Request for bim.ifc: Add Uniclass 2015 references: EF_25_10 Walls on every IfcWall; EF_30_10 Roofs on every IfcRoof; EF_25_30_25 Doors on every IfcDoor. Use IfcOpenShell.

First a look at what the model holds.

```python
import ifcopenshell

model = ifcopenshell.open("bim.ifc")
print(model.schema)
print("classifications:", [c.Name for c in model.by_type("IfcClassification")])
for ifc_class in ("IfcDoor", "IfcRoof", "IfcStair", "IfcWall", "IfcWindow"):
    print(ifc_class, len(model.by_type(ifc_class)))
```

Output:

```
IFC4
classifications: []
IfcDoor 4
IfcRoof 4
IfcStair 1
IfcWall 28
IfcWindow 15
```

```python
import ifcopenshell
import ifcopenshell.api.classification

model = ifcopenshell.open("bim.ifc")

system = ifcopenshell.api.classification.add_classification(model, classification="Uniclass 2015")

codes = {
    "IfcWall": ("EF_25_10", "Walls"),
    "IfcRoof": ("EF_30_10", "Roofs"),
    "IfcDoor": ("EF_25_30_25", "Doors"),
}
for ifc_class, (code, name) in codes.items():
    products = model.by_type(ifc_class)
    ifcopenshell.api.classification.add_reference(
        model, products=products, classification=system, identification=code, name=name
    )
    print(code, len(products))

model.write("bim_updated.ifc")
```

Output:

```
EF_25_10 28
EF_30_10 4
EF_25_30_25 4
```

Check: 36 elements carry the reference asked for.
